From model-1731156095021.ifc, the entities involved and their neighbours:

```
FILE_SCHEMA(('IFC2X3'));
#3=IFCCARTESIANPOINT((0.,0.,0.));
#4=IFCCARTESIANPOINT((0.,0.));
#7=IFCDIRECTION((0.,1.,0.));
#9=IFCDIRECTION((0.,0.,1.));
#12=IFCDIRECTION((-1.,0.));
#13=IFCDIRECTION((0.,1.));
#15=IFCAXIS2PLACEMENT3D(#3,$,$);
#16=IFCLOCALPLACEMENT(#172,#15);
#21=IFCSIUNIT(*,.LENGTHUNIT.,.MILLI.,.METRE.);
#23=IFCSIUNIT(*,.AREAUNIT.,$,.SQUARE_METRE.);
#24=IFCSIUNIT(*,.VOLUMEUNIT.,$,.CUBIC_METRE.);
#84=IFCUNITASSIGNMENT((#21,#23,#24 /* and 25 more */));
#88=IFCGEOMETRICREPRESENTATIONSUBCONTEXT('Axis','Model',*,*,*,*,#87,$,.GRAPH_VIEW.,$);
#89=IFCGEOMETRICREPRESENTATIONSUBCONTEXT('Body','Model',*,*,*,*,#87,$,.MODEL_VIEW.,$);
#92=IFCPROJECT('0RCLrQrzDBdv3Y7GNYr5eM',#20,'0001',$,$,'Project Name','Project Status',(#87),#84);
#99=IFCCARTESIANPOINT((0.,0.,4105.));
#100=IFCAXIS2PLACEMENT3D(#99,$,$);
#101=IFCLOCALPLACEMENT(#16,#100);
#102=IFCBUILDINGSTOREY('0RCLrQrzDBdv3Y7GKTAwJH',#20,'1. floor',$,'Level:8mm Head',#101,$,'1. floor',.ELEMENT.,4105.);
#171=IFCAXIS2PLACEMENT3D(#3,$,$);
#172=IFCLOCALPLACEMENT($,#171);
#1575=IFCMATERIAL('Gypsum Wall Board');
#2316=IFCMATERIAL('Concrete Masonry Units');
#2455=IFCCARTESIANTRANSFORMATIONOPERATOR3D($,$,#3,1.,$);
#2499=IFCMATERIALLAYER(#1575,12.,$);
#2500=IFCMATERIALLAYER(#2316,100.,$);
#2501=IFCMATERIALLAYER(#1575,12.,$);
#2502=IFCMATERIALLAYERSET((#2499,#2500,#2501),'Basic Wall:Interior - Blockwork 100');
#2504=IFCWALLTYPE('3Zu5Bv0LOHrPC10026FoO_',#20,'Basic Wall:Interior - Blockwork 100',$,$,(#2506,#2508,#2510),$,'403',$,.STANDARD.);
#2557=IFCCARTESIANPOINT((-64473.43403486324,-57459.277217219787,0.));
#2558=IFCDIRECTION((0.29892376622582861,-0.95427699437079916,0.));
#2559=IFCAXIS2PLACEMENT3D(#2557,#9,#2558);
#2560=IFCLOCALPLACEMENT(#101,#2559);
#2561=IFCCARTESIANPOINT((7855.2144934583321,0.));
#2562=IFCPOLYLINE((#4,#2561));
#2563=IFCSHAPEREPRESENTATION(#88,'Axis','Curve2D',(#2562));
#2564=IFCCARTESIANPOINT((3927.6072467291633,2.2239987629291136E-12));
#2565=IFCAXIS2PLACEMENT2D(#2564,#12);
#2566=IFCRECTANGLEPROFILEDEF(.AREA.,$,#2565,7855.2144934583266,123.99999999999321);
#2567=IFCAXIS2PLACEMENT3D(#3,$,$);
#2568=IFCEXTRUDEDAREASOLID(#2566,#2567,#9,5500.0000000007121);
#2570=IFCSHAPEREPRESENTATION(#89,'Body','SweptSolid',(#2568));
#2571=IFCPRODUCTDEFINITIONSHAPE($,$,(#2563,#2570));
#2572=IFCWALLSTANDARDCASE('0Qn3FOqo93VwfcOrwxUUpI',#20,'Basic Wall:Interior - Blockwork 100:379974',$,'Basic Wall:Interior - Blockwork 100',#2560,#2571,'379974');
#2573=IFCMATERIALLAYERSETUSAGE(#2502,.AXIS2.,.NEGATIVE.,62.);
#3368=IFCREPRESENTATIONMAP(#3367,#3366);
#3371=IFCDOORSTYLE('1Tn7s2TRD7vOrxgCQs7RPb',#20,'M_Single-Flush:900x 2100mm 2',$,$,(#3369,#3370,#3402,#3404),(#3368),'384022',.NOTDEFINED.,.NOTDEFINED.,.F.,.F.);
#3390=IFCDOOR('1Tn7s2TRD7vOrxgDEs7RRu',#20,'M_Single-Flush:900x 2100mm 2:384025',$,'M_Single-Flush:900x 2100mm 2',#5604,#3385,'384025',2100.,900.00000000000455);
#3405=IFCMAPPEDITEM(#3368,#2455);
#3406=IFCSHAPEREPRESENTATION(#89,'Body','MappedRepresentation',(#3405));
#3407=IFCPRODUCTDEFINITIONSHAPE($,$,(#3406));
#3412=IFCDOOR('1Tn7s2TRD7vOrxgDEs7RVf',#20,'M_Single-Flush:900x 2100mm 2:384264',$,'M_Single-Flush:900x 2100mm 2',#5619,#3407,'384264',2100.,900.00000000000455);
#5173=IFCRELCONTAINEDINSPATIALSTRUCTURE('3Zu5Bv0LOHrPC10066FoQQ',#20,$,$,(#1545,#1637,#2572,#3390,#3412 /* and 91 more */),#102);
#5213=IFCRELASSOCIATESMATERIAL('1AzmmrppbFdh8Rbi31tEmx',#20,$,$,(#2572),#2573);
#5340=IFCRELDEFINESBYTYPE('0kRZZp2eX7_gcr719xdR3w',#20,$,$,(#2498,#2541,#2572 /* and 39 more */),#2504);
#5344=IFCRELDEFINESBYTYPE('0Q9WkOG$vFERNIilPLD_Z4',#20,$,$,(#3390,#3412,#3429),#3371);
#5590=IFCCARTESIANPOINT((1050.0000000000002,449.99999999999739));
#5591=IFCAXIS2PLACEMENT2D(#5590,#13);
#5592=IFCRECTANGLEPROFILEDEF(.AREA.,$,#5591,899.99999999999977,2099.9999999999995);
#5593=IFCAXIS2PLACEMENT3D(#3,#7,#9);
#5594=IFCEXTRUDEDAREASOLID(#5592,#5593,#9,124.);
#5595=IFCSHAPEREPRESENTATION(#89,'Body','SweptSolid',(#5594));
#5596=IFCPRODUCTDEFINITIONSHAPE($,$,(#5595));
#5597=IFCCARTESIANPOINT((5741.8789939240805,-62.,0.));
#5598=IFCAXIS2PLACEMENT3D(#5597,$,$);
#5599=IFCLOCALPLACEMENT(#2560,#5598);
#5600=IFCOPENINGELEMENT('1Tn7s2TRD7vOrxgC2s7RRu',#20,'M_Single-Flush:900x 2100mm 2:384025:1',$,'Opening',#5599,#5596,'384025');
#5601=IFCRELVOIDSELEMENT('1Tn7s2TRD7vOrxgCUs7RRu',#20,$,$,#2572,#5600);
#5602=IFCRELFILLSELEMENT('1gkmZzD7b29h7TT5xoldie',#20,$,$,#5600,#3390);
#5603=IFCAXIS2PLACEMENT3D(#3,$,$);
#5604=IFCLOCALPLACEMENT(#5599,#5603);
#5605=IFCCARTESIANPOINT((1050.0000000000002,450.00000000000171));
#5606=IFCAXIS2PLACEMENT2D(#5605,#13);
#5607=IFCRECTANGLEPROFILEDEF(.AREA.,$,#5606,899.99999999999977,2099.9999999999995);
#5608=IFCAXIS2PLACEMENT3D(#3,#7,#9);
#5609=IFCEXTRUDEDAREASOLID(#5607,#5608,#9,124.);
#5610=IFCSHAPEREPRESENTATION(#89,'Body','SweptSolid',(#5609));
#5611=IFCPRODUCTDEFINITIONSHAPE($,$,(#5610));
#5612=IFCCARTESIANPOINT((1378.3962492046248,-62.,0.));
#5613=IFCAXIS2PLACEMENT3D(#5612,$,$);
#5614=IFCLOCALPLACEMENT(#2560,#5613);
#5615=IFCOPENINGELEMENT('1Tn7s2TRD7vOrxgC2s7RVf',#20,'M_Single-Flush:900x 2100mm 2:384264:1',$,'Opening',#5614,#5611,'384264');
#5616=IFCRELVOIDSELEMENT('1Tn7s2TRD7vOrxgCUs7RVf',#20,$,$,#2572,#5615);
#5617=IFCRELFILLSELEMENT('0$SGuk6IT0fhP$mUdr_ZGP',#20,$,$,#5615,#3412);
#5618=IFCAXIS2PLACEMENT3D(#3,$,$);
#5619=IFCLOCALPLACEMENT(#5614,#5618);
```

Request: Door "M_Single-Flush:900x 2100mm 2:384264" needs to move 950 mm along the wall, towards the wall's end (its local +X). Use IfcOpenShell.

```python
import ifcopenshell
import ifcopenshell.api.geometry
import ifcopenshell.util.placement
import ifcopenshell.util.unit

model = ifcopenshell.open("model-1731156095021.ifc")
unit_scale = ifcopenshell.util.unit.calculate_unit_scale(model)

door = model.by_guid("1Tn7s2TRD7vOrxgDEs7RVf")
opening = door.FillsVoids[0].RelatingOpeningElement
wall = opening.VoidsElements[0].RelatingBuildingElement

wall_matrix = ifcopenshell.util.placement.get_local_placement(wall.ObjectPlacement)
shift = wall_matrix[:3, 0] * 0.95 / unit_scale
before = ifcopenshell.util.placement.get_local_placement(door.ObjectPlacement)[:3, 3].copy()

# The door is placed relative to its opening, so it follows when the opening moves.
matrix = ifcopenshell.util.placement.get_local_placement(opening.ObjectPlacement)
matrix[:3, 3] += shift
ifcopenshell.api.geometry.edit_object_placement(
    model, product=opening, matrix=matrix, is_si=False, should_transform_children=True
)

after = ifcopenshell.util.placement.get_local_placement(door.ObjectPlacement)[:3, 3]
print("door moved by", (after - before).round(3) + 0.0)

model.write("model-1731156095021_v2.ifc")
```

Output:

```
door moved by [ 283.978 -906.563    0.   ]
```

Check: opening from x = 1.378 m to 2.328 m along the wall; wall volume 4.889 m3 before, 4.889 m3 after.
